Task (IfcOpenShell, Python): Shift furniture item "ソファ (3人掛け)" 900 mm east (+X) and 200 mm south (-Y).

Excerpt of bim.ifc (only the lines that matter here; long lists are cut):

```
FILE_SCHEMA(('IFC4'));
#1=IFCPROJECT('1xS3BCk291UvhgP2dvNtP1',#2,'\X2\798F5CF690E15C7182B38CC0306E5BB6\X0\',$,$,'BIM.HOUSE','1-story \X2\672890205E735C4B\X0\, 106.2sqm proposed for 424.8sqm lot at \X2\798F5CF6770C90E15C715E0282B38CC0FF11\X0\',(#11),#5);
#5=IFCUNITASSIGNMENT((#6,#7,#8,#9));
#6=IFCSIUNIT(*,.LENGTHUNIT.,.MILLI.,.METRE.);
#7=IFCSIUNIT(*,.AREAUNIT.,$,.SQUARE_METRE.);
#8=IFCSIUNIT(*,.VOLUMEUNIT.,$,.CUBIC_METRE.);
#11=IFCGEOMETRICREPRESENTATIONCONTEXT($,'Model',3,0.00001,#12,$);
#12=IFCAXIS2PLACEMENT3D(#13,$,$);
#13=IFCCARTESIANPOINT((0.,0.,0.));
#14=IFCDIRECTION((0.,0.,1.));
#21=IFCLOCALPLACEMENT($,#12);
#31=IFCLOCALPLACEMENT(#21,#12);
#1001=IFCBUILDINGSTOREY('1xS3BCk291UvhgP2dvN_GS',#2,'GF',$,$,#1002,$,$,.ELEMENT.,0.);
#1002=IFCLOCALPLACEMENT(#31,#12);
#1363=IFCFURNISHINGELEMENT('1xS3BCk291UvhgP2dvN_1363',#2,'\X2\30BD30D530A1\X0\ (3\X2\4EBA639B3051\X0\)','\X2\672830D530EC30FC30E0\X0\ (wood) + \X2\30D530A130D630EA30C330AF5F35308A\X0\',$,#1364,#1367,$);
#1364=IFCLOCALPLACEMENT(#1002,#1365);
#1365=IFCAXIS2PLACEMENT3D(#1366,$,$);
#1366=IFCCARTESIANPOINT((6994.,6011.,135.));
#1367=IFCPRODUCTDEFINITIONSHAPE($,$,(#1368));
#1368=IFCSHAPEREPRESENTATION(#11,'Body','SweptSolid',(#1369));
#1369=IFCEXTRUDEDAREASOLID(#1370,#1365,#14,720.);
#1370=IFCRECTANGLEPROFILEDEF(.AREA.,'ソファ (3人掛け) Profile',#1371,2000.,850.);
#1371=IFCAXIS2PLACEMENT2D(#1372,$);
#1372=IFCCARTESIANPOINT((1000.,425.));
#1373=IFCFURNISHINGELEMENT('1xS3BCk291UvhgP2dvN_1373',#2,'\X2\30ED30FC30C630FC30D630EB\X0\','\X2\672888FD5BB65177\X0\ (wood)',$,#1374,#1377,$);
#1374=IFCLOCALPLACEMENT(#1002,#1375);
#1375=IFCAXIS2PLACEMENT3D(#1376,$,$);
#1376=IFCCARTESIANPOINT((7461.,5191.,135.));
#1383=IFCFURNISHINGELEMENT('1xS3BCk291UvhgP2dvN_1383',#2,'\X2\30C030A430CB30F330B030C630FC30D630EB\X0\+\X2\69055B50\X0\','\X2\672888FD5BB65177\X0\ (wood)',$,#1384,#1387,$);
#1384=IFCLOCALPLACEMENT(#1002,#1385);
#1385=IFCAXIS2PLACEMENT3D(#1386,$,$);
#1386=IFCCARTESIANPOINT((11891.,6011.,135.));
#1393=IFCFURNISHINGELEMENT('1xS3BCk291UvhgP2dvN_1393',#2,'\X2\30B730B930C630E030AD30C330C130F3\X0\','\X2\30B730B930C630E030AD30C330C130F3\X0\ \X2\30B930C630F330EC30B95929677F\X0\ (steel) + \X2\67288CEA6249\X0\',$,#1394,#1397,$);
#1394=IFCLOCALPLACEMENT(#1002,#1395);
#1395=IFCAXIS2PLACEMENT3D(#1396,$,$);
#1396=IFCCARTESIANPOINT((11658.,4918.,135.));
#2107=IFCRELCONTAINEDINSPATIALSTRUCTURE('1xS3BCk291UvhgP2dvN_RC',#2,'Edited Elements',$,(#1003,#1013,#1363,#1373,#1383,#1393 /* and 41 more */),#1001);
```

```python
import ifcopenshell
import ifcopenshell.api.geometry
import ifcopenshell.util.placement
import ifcopenshell.util.unit

model = ifcopenshell.open("bim.ifc")
unit_scale = ifcopenshell.util.unit.calculate_unit_scale(model)

item = model.by_id(1363)
matrix = ifcopenshell.util.placement.get_local_placement(item.ObjectPlacement)
matrix[0, 3] += 0.9 / unit_scale
matrix[1, 3] -= 0.2 / unit_scale
ifcopenshell.api.geometry.edit_object_placement(model, product=item, matrix=matrix, is_si=False)

print(ifcopenshell.util.placement.get_local_placement(item.ObjectPlacement).round(3) + 0.0)

model.write("bim_edited.ifc")
```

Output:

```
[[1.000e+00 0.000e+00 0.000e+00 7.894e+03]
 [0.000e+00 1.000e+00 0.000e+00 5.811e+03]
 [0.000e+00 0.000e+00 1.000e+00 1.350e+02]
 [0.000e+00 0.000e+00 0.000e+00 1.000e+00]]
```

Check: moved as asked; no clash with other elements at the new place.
